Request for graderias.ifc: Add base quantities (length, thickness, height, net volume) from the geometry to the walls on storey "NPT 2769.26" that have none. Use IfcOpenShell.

First a look at what the model holds.

```python
import ifcopenshell
import ifcopenshell.util.element
import ifcopenshell.util.unit

model = ifcopenshell.open("graderias.ifc")
print(model.schema)
for unit_type in ("LENGTHUNIT", "AREAUNIT", "VOLUMEUNIT"):
    print(unit_type, ifcopenshell.util.unit.calculate_unit_scale(model, unit_type))
storey = next(s for s in model.by_type("IfcBuildingStorey") if s.Name == "NPT 2769.26")
walls = [e for e in ifcopenshell.util.element.get_decomposition(storey) if e.is_a("IfcWall")]
for e in sorted(walls, key=lambda e: e.id()):
    print(e.id(), e.is_a(), e.Name, list(ifcopenshell.util.element.get_psets(e, qtos_only=True)), sep=" | ")
```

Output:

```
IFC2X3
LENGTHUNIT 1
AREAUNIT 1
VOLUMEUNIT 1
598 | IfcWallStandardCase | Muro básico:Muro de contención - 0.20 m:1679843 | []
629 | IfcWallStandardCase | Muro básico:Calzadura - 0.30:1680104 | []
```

```python
import ifcopenshell
import ifcopenshell.api.pset
import ifcopenshell.geom
import ifcopenshell.util.element
import ifcopenshell.util.shape
import ifcopenshell.util.unit

model = ifcopenshell.open("graderias.ifc")
unit_scale = ifcopenshell.util.unit.calculate_unit_scale(model)
volume_scale = ifcopenshell.util.unit.calculate_unit_scale(model, "VOLUMEUNIT")
settings = ifcopenshell.geom.settings()

storey = next(s for s in model.by_type("IfcBuildingStorey") if s.Name == "NPT 2769.26")
walls = [e for e in ifcopenshell.util.element.get_decomposition(storey) if e.is_a("IfcWall")]

for e in sorted(walls, key=lambda e: e.id()):
    if ifcopenshell.util.element.get_psets(e, qtos_only=True, should_inherit=False):
        continue
    # Geometry comes back in metres, in the element's own axes.
    shape = ifcopenshell.geom.create_shape(settings, e)
    values = {
        "Length": ifcopenshell.util.shape.get_x(shape.geometry) / unit_scale,
        "Width": ifcopenshell.util.shape.get_y(shape.geometry) / unit_scale,
        "Height": ifcopenshell.util.shape.get_z(shape.geometry) / unit_scale,
        "NetVolume": ifcopenshell.util.shape.get_volume(shape.geometry) / volume_scale,
    }
    qto = ifcopenshell.api.pset.add_qto(model, product=e, name="BaseQuantities")
    ifcopenshell.api.pset.edit_qto(model, qto=qto, properties=values)
    print(e.id(), {k: round(v, 3) for k, v in values.items()})

model.write("graderias_edited.ifc")
```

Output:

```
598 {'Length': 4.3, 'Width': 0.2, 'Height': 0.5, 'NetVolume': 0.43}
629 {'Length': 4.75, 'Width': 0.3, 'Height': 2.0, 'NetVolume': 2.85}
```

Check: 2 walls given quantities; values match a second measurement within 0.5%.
